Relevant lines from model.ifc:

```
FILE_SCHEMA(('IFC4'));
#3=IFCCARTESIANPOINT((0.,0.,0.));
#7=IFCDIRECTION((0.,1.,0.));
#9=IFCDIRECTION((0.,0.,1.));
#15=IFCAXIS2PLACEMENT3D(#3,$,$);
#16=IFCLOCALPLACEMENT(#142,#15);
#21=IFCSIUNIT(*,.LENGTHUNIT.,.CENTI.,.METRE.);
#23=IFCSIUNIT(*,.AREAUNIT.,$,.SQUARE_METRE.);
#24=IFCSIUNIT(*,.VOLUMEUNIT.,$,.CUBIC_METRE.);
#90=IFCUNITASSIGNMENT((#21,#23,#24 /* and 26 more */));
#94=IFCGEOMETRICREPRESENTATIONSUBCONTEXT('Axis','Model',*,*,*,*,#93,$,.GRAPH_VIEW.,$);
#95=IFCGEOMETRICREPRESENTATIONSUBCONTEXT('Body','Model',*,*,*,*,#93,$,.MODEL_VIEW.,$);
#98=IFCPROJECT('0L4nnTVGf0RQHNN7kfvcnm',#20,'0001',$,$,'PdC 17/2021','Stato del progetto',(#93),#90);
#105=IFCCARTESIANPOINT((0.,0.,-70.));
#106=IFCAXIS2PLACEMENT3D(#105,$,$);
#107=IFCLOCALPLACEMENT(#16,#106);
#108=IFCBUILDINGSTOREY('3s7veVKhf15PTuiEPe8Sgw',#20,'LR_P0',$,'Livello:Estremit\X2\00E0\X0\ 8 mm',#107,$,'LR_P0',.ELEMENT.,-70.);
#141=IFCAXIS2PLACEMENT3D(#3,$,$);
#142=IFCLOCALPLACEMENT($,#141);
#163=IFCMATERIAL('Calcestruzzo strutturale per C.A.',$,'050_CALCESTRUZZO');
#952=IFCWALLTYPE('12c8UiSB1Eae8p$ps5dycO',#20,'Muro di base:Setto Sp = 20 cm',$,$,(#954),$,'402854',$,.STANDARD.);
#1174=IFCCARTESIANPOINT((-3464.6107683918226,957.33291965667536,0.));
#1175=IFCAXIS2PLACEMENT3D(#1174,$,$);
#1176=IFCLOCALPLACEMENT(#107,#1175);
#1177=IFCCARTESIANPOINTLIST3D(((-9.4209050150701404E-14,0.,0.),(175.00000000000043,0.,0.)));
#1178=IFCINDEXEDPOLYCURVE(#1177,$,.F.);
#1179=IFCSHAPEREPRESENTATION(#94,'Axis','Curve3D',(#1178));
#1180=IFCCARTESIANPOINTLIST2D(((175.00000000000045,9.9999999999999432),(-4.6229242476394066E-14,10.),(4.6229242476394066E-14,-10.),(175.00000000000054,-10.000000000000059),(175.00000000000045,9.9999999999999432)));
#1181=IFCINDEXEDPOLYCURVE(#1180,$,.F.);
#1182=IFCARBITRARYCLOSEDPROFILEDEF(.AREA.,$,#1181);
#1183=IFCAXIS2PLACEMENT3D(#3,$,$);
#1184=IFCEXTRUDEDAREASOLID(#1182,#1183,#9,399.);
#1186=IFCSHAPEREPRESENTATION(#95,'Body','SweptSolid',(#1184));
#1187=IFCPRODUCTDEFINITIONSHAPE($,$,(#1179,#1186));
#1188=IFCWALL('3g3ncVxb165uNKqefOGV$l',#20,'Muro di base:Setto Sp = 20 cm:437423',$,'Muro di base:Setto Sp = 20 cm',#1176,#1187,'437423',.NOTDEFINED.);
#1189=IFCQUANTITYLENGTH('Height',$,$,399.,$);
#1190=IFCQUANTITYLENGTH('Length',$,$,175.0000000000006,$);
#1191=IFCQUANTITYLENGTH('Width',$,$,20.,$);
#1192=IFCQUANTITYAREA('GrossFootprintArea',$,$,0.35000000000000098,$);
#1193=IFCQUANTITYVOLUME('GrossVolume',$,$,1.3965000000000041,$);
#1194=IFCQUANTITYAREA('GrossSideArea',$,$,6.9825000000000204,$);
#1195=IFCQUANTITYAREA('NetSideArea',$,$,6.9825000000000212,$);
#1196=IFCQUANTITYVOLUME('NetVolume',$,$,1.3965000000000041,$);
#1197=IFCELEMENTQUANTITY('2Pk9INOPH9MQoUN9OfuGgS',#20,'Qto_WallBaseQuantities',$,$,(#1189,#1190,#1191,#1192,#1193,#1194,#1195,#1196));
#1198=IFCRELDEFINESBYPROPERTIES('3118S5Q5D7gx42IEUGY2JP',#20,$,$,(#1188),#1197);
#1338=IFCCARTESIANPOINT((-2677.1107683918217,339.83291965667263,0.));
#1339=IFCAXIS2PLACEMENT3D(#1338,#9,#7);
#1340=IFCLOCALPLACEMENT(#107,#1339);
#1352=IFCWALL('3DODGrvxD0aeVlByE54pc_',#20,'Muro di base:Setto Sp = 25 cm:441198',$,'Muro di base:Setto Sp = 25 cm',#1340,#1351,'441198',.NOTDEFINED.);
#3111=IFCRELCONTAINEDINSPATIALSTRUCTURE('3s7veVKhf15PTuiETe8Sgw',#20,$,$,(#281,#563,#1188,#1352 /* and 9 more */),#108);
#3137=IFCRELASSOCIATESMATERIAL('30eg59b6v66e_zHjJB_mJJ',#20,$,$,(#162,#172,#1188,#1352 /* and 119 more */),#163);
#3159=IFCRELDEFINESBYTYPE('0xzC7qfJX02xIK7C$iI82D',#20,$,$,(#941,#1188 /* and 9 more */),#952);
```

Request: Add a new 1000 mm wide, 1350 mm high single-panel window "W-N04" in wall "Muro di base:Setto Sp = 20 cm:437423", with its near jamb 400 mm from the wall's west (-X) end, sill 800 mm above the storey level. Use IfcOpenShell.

```python
import numpy as np
import ifcopenshell
import ifcopenshell.api.feature
import ifcopenshell.api.geometry
import ifcopenshell.api.pset
import ifcopenshell.api.root
import ifcopenshell.api.spatial
import ifcopenshell.geom
import ifcopenshell.util.element
import ifcopenshell.util.placement
import ifcopenshell.util.representation
import ifcopenshell.util.shape
import ifcopenshell.util.unit

model = ifcopenshell.open("model.ifc")
unit_scale = ifcopenshell.util.unit.calculate_unit_scale(model)
area_scale = ifcopenshell.util.unit.calculate_unit_scale(model, "AREAUNIT")
volume_scale = ifcopenshell.util.unit.calculate_unit_scale(model, "VOLUMEUNIT")
settings = ifcopenshell.geom.settings()


def volume(element):
    """Net volume in cubic metres, openings subtracted."""
    shape = ifcopenshell.geom.create_shape(settings, element)
    return ifcopenshell.util.shape.get_volume(shape.geometry)


wall = model.by_id(1188)
storey = ifcopenshell.util.element.get_container(wall, ifc_class="IfcBuildingStorey")
context = ifcopenshell.util.representation.get_context(model, "Model", "Body", "MODEL_VIEW")
before = volume(wall)

width, height, from_end, sill = 1, 1.35, 0.4, 0.8  # metres

# The wall runs along its own X axis, and the end named is its -X end.
wall_shape = ifcopenshell.geom.create_shape(settings, wall)
x, y, z = ifcopenshell.util.shape.get_vertices(wall_shape.geometry).T
start = x.min() + from_end
face, thickness = float(y.min()), float(y.max() - y.min())
wall_matrix = ifcopenshell.util.placement.get_local_placement(wall.ObjectPlacement)
level = ifcopenshell.util.placement.get_local_placement(storey.ObjectPlacement)[2, 3]


def in_wall(x, y):
    """Placement at x, y metres in the wall's axes, at sill height."""
    matrix = wall_matrix.copy()
    matrix[:, 3] = wall_matrix @ np.array([x / unit_scale, y / unit_scale, 0.0, 1.0])
    matrix[2, 3] = level + sill / unit_scale
    return matrix


# Opening: a box that overshoots both wall faces by 50 mm.
opening = ifcopenshell.api.root.create_entity(model, ifc_class="IfcOpeningElement", predefined_type="OPENING")
box = ifcopenshell.api.geometry.add_wall_representation(
    model, context=context, length=width, height=height, thickness=thickness + 0.1
)
ifcopenshell.api.geometry.assign_representation(model, product=opening, representation=box)
ifcopenshell.api.geometry.edit_object_placement(model, product=opening, matrix=in_wall(start, face - 0.05), is_si=False)
ifcopenshell.api.feature.add_feature(model, feature=opening, element=wall)

window = ifcopenshell.api.root.create_entity(model, ifc_class="IfcWindow", name="W-N04", predefined_type="WINDOW")
window.OverallWidth, window.OverallHeight = width / unit_scale, height / unit_scale
window.PartitioningType = "SINGLE_PANEL"
body = ifcopenshell.api.geometry.add_window_representation(
    model,
    context=context,
    overall_width=window.OverallWidth,
    overall_height=window.OverallHeight,
    partition_type="SINGLE_PANEL",
)
ifcopenshell.api.geometry.assign_representation(model, product=window, representation=body)
ifcopenshell.api.spatial.assign_container(model, products=[window], relating_structure=storey)
ifcopenshell.api.feature.add_filling(model, opening=opening, element=window)

# Centre the window in the wall's thickness.
ifcopenshell.api.geometry.edit_object_placement(model, product=window, matrix=in_wall(start, face), is_si=False)
window_shape = ifcopenshell.geom.create_shape(settings, window)
depth = ifcopenshell.util.shape.get_vertices(window_shape.geometry)[:, 1]
offset = face + thickness / 2 - (depth.min() + depth.max()) / 2
ifcopenshell.api.geometry.edit_object_placement(model, product=window, matrix=in_wall(start, offset), is_si=False)

after = volume(wall)

# Update the wall's stored quantities.
qto = model.by_id(ifcopenshell.util.element.get_pset(wall, "Qto_WallBaseQuantities", should_inherit=False)["id"])
ifcopenshell.api.pset.edit_qto(model, qto=qto, properties={
    "NetSideArea": after / thickness / area_scale,
    "NetVolume": after / volume_scale,
})

print(f"wall volume {before:.3f} -> {after:.3f} m3")

model.write("model-out.ifc")
```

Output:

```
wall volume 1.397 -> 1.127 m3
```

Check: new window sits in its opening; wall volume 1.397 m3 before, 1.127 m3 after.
